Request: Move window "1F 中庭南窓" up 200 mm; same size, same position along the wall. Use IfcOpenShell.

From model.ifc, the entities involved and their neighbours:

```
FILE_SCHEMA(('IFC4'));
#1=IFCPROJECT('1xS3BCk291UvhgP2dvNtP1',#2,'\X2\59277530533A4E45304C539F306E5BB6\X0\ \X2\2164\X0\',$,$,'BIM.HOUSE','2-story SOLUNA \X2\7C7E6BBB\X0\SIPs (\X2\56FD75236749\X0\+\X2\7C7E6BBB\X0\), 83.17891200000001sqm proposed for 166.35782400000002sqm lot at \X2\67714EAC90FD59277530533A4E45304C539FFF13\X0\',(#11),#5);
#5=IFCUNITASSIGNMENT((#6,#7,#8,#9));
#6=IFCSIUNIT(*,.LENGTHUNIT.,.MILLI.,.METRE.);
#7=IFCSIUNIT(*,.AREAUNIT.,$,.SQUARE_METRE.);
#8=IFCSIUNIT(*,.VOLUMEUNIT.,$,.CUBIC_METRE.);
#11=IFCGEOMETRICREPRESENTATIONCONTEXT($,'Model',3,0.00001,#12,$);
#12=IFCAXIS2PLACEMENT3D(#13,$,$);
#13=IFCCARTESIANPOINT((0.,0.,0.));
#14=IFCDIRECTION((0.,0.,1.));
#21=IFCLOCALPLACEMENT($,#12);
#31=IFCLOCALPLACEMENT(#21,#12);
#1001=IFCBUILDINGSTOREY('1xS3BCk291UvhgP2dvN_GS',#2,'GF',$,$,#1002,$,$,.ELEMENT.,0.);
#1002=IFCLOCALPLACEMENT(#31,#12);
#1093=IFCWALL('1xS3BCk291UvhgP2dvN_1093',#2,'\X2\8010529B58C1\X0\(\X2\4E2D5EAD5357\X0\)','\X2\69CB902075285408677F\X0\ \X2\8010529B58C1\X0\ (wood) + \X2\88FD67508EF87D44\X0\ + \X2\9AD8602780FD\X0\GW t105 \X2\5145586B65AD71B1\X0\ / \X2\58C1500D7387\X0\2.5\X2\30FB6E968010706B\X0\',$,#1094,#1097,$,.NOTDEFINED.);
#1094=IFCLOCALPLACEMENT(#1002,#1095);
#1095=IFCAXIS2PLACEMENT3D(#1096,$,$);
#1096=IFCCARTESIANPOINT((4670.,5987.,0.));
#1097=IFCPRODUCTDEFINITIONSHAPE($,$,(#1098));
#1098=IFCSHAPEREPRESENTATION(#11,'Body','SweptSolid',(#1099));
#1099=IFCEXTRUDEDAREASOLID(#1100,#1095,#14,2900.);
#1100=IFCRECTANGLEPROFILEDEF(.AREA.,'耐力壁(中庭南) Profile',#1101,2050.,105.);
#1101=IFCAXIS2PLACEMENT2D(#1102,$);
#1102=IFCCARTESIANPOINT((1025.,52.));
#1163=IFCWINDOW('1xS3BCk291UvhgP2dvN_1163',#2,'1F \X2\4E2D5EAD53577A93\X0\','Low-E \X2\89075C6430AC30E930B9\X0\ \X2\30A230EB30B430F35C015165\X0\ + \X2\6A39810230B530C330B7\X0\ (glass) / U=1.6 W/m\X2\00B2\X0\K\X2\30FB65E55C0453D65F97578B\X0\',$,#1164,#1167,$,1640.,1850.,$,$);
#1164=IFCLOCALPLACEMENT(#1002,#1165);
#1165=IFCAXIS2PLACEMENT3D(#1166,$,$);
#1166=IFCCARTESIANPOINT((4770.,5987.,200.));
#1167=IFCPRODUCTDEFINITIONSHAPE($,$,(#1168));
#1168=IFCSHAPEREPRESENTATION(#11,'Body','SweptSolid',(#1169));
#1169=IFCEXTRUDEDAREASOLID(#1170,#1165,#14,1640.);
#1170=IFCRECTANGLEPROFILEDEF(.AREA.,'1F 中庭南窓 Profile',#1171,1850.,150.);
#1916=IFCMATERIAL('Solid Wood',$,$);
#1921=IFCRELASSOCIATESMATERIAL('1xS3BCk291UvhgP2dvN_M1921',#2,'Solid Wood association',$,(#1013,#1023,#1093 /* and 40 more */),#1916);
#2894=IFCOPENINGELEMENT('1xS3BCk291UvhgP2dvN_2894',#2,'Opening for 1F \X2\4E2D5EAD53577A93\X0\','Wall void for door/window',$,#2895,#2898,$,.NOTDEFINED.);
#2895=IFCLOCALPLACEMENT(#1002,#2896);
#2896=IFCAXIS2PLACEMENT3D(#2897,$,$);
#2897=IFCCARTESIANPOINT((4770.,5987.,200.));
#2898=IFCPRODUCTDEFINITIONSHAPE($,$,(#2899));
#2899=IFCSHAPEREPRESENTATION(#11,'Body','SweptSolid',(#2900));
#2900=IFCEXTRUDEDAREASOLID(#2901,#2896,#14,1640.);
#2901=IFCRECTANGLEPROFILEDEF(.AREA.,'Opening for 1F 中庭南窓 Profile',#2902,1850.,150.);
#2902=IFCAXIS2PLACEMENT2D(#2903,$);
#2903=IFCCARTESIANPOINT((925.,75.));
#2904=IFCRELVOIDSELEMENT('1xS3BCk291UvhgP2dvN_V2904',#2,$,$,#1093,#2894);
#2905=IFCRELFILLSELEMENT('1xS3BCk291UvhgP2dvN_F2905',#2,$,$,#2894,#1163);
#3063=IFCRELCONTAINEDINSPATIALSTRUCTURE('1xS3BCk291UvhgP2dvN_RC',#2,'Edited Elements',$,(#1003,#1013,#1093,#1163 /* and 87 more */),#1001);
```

```python
import numpy as np
import ifcopenshell
import ifcopenshell.api.geometry
import ifcopenshell.util.placement
import ifcopenshell.util.unit

model = ifcopenshell.open("model.ifc")
unit_scale = ifcopenshell.util.unit.calculate_unit_scale(model)

window = model.by_id(1163)
opening = window.FillsVoids[0].RelatingOpeningElement
dz = 200.0

shift = np.array([0.0, 0.0, dz])
# The window is not placed relative to its opening, so move both.
for product in (opening, window):
    matrix = ifcopenshell.util.placement.get_local_placement(product.ObjectPlacement)
    matrix[:3, 3] += shift
    ifcopenshell.api.geometry.edit_object_placement(model, product=product, matrix=matrix, is_si=False)

print(f"moved by {dz * unit_scale:+.3f} m")

model.write("model_updated.ifc")
```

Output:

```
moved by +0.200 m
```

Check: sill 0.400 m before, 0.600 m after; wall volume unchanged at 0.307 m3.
